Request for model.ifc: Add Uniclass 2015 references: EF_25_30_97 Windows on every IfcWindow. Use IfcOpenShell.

First a look at what the model holds.

```python
import ifcopenshell

model = ifcopenshell.open("model.ifc")
print(model.schema)
print("classifications:", [c.Name for c in model.by_type("IfcClassification")])
for ifc_class in ("IfcDoor", "IfcRoof", "IfcStair", "IfcWall", "IfcWindow"):
    print(ifc_class, len(model.by_type(ifc_class)))
```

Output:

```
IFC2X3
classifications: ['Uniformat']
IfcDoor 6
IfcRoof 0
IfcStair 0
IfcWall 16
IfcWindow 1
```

```python
import ifcopenshell
import ifcopenshell.api.classification

model = ifcopenshell.open("model.ifc")

# IFC2X3 requires Source and Edition and has no link from the project to the system.
system = model.create_entity("IfcClassification", Source="NBS", Edition="2015", Name="Uniclass 2015")

codes = {
    "IfcWindow": ("EF_25_30_97", "Windows"),
}
for ifc_class, (code, name) in codes.items():
    products = model.by_type(ifc_class)
    ifcopenshell.api.classification.add_reference(
        model, products=products, classification=system, identification=code, name=name
    )
    print(code, len(products))

model.write("model_v2.ifc")
```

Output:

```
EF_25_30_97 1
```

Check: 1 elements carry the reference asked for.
